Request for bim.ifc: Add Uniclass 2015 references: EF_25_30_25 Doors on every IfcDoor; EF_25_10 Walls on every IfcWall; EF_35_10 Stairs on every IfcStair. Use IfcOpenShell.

First a look at what the model holds.

```python
import ifcopenshell

model = ifcopenshell.open("bim.ifc")
print(model.schema)
print("classifications:", [c.Name for c in model.by_type("IfcClassification")])
for ifc_class in ("IfcDoor", "IfcRoof", "IfcStair", "IfcWall", "IfcWindow"):
    print(ifc_class, len(model.by_type(ifc_class)))
```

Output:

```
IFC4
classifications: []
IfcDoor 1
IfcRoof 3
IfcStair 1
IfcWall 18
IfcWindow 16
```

```python
import ifcopenshell
import ifcopenshell.api.classification

model = ifcopenshell.open("bim.ifc")

system = ifcopenshell.api.classification.add_classification(model, classification="Uniclass 2015")

codes = {
    "IfcDoor": ("EF_25_30_25", "Doors"),
    "IfcWall": ("EF_25_10", "Walls"),
    "IfcStair": ("EF_35_10", "Stairs"),
}
for ifc_class, (code, name) in codes.items():
    products = model.by_type(ifc_class)
    ifcopenshell.api.classification.add_reference(
        model, products=products, classification=system, identification=code, name=name
    )
    print(code, len(products))

model.write("bim_rev.ifc")
```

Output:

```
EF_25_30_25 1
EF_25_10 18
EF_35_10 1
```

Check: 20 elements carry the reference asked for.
